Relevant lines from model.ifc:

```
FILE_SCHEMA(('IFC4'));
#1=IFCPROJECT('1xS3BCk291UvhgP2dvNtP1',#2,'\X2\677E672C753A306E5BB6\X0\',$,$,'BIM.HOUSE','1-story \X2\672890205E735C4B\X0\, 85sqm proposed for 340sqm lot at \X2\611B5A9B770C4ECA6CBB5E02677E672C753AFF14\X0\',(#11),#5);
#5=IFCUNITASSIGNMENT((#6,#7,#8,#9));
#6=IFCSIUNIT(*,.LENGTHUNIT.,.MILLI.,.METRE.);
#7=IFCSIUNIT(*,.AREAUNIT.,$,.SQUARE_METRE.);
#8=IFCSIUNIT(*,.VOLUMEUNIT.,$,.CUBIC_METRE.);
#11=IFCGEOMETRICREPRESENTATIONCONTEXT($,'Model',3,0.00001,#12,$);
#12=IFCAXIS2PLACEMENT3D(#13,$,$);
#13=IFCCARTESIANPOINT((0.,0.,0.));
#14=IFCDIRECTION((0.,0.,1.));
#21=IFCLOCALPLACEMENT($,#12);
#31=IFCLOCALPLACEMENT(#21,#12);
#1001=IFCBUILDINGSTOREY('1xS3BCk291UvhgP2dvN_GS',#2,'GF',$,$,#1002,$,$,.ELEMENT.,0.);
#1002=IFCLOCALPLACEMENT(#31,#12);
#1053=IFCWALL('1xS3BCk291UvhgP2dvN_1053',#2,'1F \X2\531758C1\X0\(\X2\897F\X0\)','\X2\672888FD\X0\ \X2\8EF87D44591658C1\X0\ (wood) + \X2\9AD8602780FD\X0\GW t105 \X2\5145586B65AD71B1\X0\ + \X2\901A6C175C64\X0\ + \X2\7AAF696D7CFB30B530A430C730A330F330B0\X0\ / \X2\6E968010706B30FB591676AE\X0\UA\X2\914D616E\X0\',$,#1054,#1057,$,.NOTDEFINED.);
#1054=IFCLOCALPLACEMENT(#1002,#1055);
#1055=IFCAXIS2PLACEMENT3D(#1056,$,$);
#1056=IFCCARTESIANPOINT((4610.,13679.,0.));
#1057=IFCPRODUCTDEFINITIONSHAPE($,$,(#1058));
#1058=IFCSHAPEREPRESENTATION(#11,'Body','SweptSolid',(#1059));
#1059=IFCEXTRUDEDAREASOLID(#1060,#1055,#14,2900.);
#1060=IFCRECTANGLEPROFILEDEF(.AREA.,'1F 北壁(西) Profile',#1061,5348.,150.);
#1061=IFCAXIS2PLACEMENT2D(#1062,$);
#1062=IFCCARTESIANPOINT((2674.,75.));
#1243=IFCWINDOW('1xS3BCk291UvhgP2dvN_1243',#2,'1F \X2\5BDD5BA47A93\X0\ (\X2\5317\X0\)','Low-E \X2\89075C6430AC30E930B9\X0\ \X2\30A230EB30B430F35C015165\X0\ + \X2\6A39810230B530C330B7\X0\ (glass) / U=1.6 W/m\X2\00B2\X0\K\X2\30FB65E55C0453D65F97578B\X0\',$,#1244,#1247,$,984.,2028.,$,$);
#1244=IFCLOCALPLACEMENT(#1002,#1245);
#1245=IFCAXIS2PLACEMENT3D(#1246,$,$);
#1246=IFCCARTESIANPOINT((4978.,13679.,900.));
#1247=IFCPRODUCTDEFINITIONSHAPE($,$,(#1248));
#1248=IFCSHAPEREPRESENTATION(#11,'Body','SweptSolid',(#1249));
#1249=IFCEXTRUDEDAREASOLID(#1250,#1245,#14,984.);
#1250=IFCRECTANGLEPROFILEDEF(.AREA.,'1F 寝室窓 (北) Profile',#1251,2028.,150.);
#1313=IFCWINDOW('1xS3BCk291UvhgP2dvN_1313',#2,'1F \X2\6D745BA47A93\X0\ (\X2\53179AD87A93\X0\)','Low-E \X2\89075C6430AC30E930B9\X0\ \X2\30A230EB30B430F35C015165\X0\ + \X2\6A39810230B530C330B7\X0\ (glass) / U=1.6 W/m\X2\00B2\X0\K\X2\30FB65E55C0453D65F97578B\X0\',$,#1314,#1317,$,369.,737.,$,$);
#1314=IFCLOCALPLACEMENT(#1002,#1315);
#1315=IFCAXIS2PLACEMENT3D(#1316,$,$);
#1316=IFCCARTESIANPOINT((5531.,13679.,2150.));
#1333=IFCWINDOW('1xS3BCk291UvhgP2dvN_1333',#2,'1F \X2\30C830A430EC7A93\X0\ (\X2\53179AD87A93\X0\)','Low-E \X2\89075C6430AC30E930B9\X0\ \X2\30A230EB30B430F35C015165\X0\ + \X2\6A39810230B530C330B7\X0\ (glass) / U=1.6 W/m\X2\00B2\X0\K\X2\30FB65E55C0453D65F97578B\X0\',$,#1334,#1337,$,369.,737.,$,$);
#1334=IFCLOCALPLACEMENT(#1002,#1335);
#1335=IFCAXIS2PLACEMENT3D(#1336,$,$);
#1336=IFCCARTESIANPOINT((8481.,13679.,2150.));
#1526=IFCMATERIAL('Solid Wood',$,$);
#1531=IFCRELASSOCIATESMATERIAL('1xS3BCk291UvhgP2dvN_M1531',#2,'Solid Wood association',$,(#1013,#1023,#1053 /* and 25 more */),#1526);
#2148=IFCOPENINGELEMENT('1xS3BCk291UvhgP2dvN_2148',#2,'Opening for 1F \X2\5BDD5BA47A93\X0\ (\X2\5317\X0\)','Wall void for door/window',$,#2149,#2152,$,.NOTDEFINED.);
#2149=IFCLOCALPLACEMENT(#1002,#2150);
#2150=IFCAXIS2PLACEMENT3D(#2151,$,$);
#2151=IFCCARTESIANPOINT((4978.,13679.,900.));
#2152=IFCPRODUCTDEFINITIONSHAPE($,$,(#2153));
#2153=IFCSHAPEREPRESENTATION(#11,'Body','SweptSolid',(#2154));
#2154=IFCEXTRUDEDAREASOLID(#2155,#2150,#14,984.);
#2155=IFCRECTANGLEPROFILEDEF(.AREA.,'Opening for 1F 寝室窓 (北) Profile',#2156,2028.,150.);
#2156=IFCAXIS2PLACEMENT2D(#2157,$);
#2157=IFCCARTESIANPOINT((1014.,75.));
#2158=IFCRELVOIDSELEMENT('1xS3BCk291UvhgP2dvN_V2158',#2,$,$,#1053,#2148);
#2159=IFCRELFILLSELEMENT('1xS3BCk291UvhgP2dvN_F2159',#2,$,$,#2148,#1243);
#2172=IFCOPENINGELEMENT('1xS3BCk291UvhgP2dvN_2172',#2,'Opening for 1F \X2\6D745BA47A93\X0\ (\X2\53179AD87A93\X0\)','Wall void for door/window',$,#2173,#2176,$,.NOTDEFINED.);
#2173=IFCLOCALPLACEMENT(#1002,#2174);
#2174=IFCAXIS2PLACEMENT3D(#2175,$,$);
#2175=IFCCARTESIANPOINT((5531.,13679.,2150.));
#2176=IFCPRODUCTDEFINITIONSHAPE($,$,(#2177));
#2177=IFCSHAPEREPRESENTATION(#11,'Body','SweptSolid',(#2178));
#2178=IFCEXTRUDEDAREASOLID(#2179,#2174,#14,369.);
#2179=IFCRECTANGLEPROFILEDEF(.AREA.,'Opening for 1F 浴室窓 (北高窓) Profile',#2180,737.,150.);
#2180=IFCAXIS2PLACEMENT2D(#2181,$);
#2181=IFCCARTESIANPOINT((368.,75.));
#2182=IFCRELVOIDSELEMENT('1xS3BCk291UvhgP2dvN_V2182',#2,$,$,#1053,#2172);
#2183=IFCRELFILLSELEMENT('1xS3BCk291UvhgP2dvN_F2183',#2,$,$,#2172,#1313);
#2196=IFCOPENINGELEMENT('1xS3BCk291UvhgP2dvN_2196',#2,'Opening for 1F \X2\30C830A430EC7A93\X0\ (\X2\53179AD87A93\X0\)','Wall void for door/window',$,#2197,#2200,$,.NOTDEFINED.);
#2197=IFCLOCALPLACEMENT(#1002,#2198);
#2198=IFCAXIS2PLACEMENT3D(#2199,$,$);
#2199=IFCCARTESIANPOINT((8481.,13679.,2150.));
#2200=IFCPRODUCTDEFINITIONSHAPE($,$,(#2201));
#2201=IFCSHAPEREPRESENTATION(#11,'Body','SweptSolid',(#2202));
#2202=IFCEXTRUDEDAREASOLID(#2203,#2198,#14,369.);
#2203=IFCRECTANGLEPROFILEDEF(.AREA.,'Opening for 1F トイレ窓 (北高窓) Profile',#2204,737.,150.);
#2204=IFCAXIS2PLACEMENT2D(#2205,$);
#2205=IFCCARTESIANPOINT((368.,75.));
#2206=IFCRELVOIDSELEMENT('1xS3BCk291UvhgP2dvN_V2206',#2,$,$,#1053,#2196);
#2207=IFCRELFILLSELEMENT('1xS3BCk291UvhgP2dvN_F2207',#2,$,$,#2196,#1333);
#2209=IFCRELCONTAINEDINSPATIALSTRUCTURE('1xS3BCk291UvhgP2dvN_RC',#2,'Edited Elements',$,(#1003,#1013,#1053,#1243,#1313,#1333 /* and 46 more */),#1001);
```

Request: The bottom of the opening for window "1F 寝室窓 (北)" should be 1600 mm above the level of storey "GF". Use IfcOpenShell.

```python
import numpy as np
import ifcopenshell
import ifcopenshell.api.geometry
import ifcopenshell.geom
import ifcopenshell.util.element
import ifcopenshell.util.placement
import ifcopenshell.util.shape
import ifcopenshell.util.unit

model = ifcopenshell.open("model.ifc")
unit_scale = ifcopenshell.util.unit.calculate_unit_scale(model)

window = model.by_guid("1xS3BCk291UvhgP2dvN_1243")
opening = window.FillsVoids[0].RelatingOpeningElement
storey = ifcopenshell.util.element.get_container(window, ifc_class="IfcBuildingStorey")
level = ifcopenshell.util.placement.get_local_placement(storey.ObjectPlacement)[2, 3]

# The opening's origin need not be at the sill, so measure its lowest point.
shape = ifcopenshell.geom.create_shape(ifcopenshell.geom.settings(), opening)
bottom = ifcopenshell.util.shape.get_shape_bottom_elevation(shape, shape.geometry) / unit_scale
dz = level + 1600.0 - bottom

shift = np.array([0.0, 0.0, dz])
# The window is not placed relative to its opening, so move both.
for product in (opening, window):
    matrix = ifcopenshell.util.placement.get_local_placement(product.ObjectPlacement)
    matrix[:3, 3] += shift
    ifcopenshell.api.geometry.edit_object_placement(model, product=product, matrix=matrix, is_si=False)

print(f"moved by {dz * unit_scale:+.3f} m")

model.write("model_v2.ifc")
```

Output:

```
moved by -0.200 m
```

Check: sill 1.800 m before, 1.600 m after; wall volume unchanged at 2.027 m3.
